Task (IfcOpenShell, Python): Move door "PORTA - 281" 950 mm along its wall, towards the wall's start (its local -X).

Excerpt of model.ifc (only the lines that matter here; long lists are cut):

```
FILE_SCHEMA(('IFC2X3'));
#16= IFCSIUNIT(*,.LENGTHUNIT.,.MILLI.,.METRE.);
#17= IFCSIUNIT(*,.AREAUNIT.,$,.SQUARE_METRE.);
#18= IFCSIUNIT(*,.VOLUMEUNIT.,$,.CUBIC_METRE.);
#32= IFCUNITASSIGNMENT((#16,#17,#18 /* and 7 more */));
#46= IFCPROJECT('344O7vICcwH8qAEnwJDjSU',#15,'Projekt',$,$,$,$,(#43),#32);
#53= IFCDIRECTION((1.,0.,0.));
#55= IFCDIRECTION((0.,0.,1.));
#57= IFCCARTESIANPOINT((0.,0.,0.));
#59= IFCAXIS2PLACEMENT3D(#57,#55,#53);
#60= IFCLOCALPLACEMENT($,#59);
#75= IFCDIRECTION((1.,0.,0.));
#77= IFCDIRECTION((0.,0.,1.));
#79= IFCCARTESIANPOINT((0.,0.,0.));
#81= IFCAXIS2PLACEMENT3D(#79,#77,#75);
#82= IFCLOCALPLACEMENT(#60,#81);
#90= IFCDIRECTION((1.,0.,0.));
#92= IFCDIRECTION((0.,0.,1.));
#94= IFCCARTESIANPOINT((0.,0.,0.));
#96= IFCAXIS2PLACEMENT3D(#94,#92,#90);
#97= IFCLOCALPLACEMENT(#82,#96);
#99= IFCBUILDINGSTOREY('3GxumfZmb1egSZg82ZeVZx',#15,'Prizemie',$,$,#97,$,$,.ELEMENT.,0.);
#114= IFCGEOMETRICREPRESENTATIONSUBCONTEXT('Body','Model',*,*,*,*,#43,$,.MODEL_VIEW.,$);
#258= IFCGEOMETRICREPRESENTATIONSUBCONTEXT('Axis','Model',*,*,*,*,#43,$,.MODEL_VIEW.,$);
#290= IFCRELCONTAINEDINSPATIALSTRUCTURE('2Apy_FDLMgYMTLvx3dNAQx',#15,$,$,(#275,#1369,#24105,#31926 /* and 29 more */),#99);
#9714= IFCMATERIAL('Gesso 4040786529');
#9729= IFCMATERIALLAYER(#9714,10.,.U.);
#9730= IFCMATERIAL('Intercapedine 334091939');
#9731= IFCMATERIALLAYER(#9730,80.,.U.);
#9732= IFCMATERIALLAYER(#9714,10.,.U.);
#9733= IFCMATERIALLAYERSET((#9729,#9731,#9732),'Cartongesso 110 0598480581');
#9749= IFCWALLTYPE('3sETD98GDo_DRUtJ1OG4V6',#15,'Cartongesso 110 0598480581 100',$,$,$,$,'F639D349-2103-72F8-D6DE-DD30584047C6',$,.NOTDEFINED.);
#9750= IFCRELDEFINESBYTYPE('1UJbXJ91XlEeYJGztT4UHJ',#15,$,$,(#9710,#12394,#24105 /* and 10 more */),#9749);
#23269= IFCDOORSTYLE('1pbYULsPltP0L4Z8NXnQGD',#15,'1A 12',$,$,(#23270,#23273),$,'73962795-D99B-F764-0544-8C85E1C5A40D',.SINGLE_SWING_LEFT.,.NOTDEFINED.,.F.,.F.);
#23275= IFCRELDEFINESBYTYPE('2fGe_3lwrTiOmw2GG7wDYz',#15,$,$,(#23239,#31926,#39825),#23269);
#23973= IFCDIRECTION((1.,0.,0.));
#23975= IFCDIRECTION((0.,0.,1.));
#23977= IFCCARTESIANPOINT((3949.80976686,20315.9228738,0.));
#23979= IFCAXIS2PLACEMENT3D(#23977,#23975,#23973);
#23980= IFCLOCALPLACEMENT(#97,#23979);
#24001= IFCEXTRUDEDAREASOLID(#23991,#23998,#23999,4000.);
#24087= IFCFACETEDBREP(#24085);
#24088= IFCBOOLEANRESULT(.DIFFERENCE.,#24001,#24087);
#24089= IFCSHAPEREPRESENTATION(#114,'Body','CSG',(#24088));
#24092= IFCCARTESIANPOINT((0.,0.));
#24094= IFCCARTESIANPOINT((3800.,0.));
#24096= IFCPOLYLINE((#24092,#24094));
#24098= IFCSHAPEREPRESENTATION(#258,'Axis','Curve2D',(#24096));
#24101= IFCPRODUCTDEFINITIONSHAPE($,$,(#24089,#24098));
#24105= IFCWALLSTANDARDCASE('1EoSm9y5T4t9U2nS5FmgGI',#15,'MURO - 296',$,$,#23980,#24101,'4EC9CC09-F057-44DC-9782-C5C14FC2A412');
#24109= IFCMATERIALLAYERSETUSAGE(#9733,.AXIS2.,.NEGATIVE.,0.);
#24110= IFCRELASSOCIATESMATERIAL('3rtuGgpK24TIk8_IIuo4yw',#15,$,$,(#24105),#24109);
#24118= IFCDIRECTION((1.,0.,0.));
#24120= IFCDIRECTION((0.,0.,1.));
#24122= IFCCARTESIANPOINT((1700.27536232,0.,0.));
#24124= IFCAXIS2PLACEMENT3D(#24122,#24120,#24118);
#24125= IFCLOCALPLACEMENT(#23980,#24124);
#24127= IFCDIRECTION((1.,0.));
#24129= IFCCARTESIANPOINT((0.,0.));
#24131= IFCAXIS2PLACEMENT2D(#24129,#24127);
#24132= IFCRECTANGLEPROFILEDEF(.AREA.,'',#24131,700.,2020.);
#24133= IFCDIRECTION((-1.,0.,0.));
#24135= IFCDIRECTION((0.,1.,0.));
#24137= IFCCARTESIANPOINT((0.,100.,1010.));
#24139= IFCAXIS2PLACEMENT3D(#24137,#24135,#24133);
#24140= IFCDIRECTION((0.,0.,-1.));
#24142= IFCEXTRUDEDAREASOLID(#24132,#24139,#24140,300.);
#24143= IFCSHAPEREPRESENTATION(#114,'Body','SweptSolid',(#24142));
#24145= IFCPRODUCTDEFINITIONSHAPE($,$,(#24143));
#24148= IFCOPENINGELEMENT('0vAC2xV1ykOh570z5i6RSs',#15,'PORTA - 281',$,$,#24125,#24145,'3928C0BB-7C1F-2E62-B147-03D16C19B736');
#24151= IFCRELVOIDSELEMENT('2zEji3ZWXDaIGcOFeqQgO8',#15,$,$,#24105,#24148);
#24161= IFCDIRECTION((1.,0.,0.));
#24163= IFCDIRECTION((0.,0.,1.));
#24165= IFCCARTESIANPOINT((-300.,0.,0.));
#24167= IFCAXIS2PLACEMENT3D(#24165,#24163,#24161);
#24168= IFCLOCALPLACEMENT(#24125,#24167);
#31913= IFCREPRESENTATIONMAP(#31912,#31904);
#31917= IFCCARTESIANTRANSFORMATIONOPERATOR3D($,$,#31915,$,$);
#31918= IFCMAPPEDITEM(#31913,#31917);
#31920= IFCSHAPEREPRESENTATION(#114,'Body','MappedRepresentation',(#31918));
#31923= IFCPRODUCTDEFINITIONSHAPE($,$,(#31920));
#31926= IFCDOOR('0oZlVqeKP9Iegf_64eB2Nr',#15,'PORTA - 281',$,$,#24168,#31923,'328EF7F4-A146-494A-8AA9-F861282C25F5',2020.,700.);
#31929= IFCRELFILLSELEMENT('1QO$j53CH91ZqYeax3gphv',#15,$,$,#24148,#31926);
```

```python
import ifcopenshell
import ifcopenshell.api.geometry
import ifcopenshell.util.placement
import ifcopenshell.util.unit

model = ifcopenshell.open("model.ifc")
unit_scale = ifcopenshell.util.unit.calculate_unit_scale(model)

door = model.by_guid("0oZlVqeKP9Iegf_64eB2Nr")
opening = door.FillsVoids[0].RelatingOpeningElement
wall = opening.VoidsElements[0].RelatingBuildingElement

wall_matrix = ifcopenshell.util.placement.get_local_placement(wall.ObjectPlacement)
shift = wall_matrix[:3, 0] * -0.95 / unit_scale
before = ifcopenshell.util.placement.get_local_placement(door.ObjectPlacement)[:3, 3].copy()

# The door is placed relative to its opening, so it follows when the opening moves.
matrix = ifcopenshell.util.placement.get_local_placement(opening.ObjectPlacement)
matrix[:3, 3] += shift
ifcopenshell.api.geometry.edit_object_placement(
    model, product=opening, matrix=matrix, is_si=False, should_transform_children=True
)

after = ifcopenshell.util.placement.get_local_placement(door.ObjectPlacement)[:3, 3]
print("door moved by", (after - before).round(3) + 0.0)

model.write("model_updated.ifc")
```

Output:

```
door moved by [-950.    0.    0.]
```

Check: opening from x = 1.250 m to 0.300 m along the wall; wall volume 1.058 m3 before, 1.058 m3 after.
